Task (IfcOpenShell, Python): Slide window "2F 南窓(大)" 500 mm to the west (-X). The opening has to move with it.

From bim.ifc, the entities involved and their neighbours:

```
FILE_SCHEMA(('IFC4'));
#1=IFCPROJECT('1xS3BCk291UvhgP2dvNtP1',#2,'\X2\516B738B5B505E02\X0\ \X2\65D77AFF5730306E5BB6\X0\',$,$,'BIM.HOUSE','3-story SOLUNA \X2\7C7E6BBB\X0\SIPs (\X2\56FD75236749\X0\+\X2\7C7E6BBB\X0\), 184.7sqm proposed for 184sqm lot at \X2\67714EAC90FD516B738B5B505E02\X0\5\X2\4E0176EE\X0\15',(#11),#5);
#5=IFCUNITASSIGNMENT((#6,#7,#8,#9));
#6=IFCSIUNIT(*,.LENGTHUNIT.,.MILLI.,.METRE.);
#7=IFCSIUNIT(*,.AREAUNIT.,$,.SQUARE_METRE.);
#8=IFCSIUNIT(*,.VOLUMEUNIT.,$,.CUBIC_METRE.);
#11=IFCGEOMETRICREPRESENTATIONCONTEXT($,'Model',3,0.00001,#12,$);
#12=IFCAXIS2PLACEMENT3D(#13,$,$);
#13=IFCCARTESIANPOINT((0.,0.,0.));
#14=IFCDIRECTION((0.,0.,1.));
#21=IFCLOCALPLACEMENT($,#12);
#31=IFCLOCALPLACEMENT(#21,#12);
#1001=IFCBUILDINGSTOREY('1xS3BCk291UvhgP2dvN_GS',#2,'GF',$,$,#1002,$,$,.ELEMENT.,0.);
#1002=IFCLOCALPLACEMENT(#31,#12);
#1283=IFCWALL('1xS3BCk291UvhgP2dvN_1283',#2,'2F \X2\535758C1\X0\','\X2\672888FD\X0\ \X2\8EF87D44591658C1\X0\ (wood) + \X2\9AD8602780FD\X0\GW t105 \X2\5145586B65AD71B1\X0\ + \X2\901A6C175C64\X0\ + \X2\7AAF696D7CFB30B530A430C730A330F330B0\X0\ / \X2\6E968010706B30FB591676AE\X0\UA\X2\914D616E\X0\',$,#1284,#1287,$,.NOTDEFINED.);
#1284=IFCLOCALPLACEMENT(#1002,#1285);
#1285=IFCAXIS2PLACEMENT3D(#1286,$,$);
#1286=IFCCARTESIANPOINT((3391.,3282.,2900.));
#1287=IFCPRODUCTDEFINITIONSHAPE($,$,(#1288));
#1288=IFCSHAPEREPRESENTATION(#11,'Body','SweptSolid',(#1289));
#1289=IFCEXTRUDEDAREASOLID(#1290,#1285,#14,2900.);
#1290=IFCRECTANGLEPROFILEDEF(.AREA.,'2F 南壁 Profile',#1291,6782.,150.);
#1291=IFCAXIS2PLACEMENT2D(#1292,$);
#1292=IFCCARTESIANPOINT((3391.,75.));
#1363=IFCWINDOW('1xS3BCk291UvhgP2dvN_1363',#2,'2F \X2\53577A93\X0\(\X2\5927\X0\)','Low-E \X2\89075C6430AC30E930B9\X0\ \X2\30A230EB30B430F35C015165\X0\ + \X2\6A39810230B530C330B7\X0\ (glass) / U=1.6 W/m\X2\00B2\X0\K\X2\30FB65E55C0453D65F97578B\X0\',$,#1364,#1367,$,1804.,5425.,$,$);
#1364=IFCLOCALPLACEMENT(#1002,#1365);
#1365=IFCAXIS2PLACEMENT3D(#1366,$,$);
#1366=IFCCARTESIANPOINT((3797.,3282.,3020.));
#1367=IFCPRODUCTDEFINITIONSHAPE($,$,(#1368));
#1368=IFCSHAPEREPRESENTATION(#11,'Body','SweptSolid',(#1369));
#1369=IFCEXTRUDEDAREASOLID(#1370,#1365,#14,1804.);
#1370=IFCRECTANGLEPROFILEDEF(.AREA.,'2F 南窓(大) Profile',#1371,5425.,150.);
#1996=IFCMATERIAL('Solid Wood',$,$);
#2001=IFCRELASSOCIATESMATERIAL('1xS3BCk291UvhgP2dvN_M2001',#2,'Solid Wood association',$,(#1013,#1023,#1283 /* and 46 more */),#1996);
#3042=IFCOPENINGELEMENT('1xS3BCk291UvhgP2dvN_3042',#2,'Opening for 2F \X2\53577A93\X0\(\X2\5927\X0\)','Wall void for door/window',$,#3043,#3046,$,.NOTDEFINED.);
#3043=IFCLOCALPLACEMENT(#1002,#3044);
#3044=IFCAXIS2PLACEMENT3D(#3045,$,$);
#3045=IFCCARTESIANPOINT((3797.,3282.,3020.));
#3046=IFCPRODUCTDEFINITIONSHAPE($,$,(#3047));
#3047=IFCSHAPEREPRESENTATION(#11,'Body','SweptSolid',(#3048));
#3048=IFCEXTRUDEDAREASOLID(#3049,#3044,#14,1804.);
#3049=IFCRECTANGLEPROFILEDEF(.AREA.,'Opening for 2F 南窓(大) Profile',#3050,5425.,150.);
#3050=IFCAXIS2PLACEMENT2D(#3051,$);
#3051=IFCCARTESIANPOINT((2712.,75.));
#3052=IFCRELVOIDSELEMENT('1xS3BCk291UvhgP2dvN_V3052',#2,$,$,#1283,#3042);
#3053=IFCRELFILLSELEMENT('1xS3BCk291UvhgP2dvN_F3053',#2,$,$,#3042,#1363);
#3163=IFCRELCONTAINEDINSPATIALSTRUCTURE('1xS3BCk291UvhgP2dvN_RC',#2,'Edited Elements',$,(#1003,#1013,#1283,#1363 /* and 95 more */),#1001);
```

```python
import ifcopenshell
import ifcopenshell.api.geometry
import ifcopenshell.util.placement
import ifcopenshell.util.unit

model = ifcopenshell.open("bim.ifc")
unit_scale = ifcopenshell.util.unit.calculate_unit_scale(model)

window = model.by_guid("1xS3BCk291UvhgP2dvN_1363")
opening = window.FillsVoids[0].RelatingOpeningElement
wall = opening.VoidsElements[0].RelatingBuildingElement

wall_matrix = ifcopenshell.util.placement.get_local_placement(wall.ObjectPlacement)
shift = wall_matrix[:3, 0] * -0.5 / unit_scale
before = ifcopenshell.util.placement.get_local_placement(window.ObjectPlacement)[:3, 3].copy()

# The window is not placed relative to its opening, so move both.
for product in (opening, window):
    matrix = ifcopenshell.util.placement.get_local_placement(product.ObjectPlacement)
    matrix[:3, 3] += shift
    ifcopenshell.api.geometry.edit_object_placement(model, product=product, matrix=matrix, is_si=False)

after = ifcopenshell.util.placement.get_local_placement(window.ObjectPlacement)[:3, 3]
print("window moved by", (after - before).round(3) + 0.0)

model.write("bim_v2.ifc")
```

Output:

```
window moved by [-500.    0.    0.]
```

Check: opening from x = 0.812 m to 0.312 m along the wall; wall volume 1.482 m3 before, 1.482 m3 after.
